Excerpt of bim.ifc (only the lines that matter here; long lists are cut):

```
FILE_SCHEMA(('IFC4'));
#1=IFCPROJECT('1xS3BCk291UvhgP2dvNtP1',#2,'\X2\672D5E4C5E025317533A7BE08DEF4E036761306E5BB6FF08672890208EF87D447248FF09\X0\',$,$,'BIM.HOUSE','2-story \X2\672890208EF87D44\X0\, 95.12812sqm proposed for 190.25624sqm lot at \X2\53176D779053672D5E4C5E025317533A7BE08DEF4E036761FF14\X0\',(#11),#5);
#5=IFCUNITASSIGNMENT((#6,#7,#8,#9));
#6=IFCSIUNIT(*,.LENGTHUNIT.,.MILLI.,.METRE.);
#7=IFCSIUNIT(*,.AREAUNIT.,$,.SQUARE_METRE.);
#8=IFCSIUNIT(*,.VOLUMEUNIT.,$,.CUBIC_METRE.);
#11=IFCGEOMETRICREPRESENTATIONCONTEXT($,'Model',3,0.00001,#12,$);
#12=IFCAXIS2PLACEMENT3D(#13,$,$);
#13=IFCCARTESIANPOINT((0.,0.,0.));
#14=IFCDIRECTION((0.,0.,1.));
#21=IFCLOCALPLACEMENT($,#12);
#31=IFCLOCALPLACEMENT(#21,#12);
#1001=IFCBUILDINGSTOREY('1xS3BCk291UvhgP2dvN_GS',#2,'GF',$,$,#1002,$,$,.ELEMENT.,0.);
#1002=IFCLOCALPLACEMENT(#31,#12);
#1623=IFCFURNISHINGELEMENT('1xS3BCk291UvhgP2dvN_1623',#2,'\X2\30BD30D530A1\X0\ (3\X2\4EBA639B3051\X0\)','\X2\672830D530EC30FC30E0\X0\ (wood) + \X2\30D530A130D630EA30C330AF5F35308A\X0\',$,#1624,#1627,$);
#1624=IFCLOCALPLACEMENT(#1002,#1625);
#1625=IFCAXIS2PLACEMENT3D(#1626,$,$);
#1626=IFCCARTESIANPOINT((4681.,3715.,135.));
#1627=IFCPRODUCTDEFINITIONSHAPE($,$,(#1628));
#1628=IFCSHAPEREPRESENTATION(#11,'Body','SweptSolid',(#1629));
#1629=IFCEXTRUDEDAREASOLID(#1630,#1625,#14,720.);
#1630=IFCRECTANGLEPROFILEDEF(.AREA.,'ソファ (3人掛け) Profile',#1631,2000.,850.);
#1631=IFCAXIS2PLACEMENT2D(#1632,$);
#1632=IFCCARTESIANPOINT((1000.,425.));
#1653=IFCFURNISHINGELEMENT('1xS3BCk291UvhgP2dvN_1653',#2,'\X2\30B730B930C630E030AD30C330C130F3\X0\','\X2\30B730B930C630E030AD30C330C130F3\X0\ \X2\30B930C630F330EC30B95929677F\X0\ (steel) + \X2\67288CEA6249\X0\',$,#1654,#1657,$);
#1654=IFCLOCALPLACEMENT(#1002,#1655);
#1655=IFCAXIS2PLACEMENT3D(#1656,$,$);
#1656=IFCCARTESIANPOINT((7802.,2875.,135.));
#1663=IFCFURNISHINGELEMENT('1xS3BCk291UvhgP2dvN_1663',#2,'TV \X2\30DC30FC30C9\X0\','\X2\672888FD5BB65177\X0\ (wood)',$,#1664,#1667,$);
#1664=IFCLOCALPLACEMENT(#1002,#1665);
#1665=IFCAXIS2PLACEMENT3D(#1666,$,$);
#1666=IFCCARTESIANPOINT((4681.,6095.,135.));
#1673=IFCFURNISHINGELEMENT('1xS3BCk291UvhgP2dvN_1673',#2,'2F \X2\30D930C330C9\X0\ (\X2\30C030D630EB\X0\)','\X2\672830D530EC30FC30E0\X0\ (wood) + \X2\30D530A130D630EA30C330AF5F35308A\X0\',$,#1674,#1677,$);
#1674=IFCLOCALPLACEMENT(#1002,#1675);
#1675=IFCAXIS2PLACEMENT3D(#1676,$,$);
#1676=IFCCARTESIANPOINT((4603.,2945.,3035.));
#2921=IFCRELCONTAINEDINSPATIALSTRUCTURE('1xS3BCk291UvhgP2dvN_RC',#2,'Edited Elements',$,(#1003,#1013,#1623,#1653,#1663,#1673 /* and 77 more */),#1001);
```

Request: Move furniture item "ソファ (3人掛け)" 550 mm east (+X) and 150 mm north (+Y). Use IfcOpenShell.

```python
import ifcopenshell
import ifcopenshell.api.geometry
import ifcopenshell.util.placement

model = ifcopenshell.open("bim.ifc")

item = model.by_id(1623)
matrix = ifcopenshell.util.placement.get_local_placement(item.ObjectPlacement)
matrix[0, 3] += 550.0
matrix[1, 3] += 150.0
ifcopenshell.api.geometry.edit_object_placement(model, product=item, matrix=matrix, is_si=False)

print(ifcopenshell.util.placement.get_local_placement(item.ObjectPlacement).round(3) + 0.0)

model.write("bim_v2.ifc")
```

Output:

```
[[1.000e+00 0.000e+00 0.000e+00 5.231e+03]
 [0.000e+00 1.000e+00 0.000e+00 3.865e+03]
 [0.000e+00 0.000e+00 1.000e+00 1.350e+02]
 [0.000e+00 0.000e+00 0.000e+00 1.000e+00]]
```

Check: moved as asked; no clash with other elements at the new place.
